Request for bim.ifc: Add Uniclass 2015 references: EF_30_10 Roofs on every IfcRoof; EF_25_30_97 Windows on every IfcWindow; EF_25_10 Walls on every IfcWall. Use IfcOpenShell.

First a look at what the model holds.

```python
import ifcopenshell

model = ifcopenshell.open("bim.ifc")
print(model.schema)
print("classifications:", [c.Name for c in model.by_type("IfcClassification")])
for ifc_class in ("IfcDoor", "IfcRoof", "IfcStair", "IfcWall", "IfcWindow"):
    print(ifc_class, len(model.by_type(ifc_class)))
```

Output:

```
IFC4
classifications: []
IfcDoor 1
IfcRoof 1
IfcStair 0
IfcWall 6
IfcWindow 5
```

```python
import ifcopenshell
import ifcopenshell.api.classification

model = ifcopenshell.open("bim.ifc")

system = ifcopenshell.api.classification.add_classification(model, classification="Uniclass 2015")

codes = {
    "IfcRoof": ("EF_30_10", "Roofs"),
    "IfcWindow": ("EF_25_30_97", "Windows"),
    "IfcWall": ("EF_25_10", "Walls"),
}
for ifc_class, (code, name) in codes.items():
    products = model.by_type(ifc_class)
    ifcopenshell.api.classification.add_reference(
        model, products=products, classification=system, identification=code, name=name
    )
    print(code, len(products))

model.write("bim_rev.ifc")
```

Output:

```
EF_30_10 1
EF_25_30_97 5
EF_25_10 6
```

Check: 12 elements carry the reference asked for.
